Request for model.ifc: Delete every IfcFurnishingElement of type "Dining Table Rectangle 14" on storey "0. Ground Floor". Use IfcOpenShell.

First a look at what the model holds.

```python
import ifcopenshell
import ifcopenshell.util.element

model = ifcopenshell.open("model.ifc")
print(model.schema)
storey = next(s for s in model.by_type("IfcBuildingStorey") if s.Name == "0. Ground Floor")
furniture = [e for e in ifcopenshell.util.element.get_decomposition(storey) if e.is_a("IfcFurnishingElement")]
seen = {}
for e in furniture:
    element_type = ifcopenshell.util.element.get_type(e)
    name = element_type.Name if element_type not in (None, e) else None
    seen[name] = seen.get(name, 0) + 1
for name, count in sorted(seen.items(), key=str):
    print(count, "x", name)
```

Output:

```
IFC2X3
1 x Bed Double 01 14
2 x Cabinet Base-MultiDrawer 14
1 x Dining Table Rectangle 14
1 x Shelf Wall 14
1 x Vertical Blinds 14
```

```python
import ifcopenshell
import ifcopenshell.api.root
import ifcopenshell.util.element

model = ifcopenshell.open("model.ifc")

storey = next(s for s in model.by_type("IfcBuildingStorey") if s.Name == "0. Ground Floor")
furniture = [e for e in ifcopenshell.util.element.get_decomposition(storey) if e.is_a("IfcFurnishingElement")]
targets = [e for e in furniture if (t := ifcopenshell.util.element.get_type(e)) not in (None, e) and t.Name == "Dining Table Rectangle 14"]

for e in targets:
    ifcopenshell.api.root.remove_product(model, product=e)
print(len(targets), "removed")

model.write("model_rev.ifc")
```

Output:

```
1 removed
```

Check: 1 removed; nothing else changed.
